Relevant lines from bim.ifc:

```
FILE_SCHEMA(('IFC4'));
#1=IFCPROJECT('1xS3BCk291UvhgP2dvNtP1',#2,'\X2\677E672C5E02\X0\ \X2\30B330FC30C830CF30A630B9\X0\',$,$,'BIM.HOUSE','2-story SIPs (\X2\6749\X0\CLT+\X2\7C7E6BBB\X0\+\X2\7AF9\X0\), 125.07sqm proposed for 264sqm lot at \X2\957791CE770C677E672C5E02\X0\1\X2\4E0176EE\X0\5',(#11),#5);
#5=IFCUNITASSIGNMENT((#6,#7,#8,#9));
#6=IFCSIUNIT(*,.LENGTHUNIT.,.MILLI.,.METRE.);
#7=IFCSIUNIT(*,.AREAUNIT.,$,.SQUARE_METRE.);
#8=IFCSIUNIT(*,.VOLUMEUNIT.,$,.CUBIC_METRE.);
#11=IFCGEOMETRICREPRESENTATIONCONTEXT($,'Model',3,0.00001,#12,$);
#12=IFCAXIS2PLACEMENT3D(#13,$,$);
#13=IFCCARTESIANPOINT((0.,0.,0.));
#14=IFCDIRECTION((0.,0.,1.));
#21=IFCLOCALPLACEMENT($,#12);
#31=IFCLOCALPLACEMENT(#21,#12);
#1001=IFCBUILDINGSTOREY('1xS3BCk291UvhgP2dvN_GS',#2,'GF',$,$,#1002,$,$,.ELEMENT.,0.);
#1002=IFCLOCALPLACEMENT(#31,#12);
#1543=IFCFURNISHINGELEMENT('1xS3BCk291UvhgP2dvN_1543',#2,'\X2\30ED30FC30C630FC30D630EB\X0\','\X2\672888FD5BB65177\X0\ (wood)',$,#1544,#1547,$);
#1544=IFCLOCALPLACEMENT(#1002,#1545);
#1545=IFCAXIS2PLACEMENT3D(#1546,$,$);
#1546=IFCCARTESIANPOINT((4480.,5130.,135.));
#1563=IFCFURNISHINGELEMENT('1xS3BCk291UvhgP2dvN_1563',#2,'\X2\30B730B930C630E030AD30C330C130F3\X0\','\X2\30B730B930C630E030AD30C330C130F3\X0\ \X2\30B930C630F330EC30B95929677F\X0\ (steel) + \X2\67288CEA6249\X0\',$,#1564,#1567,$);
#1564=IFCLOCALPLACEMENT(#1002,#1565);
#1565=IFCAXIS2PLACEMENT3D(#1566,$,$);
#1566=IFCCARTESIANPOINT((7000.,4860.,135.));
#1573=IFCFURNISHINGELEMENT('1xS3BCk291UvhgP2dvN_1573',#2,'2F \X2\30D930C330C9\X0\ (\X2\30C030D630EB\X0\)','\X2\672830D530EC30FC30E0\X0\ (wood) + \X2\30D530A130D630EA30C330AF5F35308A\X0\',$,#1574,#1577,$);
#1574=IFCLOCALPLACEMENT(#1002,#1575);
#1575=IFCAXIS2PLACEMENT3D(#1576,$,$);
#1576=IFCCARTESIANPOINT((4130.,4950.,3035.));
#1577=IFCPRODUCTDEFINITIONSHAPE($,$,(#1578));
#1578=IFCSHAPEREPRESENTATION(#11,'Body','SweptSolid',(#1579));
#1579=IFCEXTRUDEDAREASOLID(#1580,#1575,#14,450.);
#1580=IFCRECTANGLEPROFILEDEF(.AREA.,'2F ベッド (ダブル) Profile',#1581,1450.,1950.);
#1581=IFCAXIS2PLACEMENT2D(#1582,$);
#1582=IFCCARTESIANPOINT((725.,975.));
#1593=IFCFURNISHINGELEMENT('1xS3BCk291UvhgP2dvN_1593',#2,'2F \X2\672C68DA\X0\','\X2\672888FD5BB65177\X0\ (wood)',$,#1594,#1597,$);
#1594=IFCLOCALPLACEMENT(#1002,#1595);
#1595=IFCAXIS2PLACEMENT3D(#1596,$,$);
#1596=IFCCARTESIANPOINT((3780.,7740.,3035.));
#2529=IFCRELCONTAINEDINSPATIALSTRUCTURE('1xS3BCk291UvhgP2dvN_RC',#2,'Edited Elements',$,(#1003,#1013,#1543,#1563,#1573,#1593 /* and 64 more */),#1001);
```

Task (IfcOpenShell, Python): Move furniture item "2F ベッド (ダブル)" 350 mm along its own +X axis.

```python
import ifcopenshell
import ifcopenshell.api.geometry
import ifcopenshell.util.placement
import ifcopenshell.util.unit

model = ifcopenshell.open("bim.ifc")
unit_scale = ifcopenshell.util.unit.calculate_unit_scale(model)

item = model.by_guid("1xS3BCk291UvhgP2dvN_1573")
matrix = ifcopenshell.util.placement.get_local_placement(item.ObjectPlacement)
matrix[:3, 3] += matrix[:3, 0] * 0.35 / unit_scale
ifcopenshell.api.geometry.edit_object_placement(model, product=item, matrix=matrix, is_si=False)

print(ifcopenshell.util.placement.get_local_placement(item.ObjectPlacement).round(3) + 0.0)

model.write("bim-out.ifc")
```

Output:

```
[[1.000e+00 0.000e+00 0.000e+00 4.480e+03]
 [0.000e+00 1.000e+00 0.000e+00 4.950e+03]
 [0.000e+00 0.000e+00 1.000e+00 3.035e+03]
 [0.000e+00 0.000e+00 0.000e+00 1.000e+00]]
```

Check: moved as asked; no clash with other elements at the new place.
